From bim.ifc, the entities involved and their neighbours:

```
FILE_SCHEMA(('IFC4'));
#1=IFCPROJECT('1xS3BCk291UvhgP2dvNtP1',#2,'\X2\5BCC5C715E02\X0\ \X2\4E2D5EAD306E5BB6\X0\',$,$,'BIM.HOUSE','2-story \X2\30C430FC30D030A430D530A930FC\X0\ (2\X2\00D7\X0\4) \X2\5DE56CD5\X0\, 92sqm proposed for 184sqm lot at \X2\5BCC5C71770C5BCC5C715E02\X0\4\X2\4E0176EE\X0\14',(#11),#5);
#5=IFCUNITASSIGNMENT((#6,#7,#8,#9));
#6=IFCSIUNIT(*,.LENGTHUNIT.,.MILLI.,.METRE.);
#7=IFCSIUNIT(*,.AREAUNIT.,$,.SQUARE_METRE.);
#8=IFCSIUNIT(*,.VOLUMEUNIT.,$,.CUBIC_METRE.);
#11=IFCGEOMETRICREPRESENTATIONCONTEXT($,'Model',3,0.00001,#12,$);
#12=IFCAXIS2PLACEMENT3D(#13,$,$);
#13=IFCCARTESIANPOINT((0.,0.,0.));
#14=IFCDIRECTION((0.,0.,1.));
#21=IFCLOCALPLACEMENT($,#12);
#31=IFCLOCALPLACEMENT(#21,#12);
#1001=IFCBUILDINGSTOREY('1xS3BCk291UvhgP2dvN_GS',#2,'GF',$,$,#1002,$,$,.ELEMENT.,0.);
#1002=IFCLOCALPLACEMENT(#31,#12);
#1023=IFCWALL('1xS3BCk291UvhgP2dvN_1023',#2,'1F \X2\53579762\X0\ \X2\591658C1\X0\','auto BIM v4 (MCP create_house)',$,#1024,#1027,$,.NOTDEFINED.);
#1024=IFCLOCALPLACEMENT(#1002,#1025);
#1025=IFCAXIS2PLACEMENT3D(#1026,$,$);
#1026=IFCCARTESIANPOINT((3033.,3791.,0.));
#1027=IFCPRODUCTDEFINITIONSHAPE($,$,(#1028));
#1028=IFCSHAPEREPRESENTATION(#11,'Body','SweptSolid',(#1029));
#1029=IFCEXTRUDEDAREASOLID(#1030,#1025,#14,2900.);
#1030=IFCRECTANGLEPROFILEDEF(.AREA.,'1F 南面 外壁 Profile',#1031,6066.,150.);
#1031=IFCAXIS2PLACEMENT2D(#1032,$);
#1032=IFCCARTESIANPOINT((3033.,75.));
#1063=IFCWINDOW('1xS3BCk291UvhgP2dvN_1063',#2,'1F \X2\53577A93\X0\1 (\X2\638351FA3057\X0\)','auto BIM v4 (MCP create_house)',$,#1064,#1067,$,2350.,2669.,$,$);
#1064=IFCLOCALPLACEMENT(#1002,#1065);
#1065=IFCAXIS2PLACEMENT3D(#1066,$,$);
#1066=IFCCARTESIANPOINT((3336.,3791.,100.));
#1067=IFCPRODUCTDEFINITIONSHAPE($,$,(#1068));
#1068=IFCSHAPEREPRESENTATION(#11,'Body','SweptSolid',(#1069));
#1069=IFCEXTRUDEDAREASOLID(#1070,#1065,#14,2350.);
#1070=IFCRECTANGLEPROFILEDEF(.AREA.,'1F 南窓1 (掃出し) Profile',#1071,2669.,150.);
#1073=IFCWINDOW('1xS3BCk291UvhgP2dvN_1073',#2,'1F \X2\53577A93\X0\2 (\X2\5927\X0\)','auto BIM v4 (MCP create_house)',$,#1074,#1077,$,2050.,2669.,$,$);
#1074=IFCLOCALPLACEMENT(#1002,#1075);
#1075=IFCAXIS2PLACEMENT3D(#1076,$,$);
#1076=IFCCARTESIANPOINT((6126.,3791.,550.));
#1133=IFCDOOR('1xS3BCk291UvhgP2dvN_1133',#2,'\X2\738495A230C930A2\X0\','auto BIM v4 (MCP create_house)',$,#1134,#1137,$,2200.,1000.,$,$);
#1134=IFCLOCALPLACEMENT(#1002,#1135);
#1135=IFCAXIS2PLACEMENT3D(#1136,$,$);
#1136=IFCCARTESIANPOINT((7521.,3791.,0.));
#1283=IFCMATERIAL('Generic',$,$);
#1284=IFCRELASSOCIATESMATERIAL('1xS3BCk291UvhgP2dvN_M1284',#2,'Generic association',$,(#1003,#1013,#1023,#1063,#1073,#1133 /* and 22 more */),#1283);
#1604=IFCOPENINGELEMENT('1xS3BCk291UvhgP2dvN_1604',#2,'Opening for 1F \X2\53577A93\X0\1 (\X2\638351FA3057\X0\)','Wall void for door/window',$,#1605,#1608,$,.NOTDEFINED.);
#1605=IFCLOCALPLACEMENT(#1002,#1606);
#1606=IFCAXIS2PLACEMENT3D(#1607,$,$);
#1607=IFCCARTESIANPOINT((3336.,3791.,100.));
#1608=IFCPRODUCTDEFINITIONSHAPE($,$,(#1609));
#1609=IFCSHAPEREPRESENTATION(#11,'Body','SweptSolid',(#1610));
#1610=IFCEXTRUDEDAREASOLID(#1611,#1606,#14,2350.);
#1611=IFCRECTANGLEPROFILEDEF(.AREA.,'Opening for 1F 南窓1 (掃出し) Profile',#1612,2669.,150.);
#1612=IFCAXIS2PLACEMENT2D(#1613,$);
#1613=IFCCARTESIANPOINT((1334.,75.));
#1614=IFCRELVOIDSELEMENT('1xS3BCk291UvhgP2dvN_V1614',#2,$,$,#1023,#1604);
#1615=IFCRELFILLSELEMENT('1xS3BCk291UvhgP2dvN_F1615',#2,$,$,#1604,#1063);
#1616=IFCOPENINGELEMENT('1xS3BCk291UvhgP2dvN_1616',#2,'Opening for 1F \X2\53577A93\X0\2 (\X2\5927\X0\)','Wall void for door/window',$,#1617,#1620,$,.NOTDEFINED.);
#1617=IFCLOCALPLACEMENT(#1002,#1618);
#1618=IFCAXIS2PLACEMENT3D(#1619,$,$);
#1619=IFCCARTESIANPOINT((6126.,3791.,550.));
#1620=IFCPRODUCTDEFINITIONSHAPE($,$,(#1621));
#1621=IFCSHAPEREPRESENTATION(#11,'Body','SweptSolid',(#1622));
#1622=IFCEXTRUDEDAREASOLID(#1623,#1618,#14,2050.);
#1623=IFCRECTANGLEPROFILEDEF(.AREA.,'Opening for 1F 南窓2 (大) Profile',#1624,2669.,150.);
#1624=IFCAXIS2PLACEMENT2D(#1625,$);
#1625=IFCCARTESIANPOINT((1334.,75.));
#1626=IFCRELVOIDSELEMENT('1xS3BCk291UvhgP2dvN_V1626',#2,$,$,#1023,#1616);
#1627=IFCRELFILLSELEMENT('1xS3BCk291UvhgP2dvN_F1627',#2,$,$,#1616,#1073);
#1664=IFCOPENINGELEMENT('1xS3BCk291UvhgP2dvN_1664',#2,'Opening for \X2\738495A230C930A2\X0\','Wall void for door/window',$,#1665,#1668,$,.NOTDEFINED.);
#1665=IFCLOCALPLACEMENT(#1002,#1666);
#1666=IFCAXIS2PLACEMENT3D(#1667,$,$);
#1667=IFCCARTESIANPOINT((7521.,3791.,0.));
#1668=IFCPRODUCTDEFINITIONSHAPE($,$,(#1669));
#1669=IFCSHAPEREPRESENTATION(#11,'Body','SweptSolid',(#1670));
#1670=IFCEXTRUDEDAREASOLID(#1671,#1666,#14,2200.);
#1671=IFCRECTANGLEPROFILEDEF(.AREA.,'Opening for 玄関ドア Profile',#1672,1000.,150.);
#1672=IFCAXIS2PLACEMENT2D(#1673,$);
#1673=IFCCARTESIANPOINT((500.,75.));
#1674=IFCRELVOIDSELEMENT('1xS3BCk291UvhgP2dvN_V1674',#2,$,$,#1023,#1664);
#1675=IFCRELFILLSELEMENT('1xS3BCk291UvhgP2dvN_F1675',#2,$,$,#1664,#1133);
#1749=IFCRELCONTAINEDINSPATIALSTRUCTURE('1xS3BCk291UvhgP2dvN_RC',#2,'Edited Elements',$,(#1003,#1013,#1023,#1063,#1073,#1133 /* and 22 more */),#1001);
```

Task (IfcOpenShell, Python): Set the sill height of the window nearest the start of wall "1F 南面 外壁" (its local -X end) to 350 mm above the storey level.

```python
import numpy as np
import ifcopenshell
import ifcopenshell.api.geometry
import ifcopenshell.geom
import ifcopenshell.util.element
import ifcopenshell.util.placement
import ifcopenshell.util.shape
import ifcopenshell.util.unit

model = ifcopenshell.open("bim.ifc")
unit_scale = ifcopenshell.util.unit.calculate_unit_scale(model)

window = model.by_guid("1xS3BCk291UvhgP2dvN_1063")
opening = window.FillsVoids[0].RelatingOpeningElement
storey = ifcopenshell.util.element.get_container(window, ifc_class="IfcBuildingStorey")
level = ifcopenshell.util.placement.get_local_placement(storey.ObjectPlacement)[2, 3]

# The opening's origin need not be at the sill, so measure its lowest point.
shape = ifcopenshell.geom.create_shape(ifcopenshell.geom.settings(), opening)
bottom = ifcopenshell.util.shape.get_shape_bottom_elevation(shape, shape.geometry) / unit_scale
dz = level + 0.35 / unit_scale - bottom

shift = np.array([0.0, 0.0, dz])
# The window is not placed relative to its opening, so move both.
for product in (opening, window):
    matrix = ifcopenshell.util.placement.get_local_placement(product.ObjectPlacement)
    matrix[:3, 3] += shift
    ifcopenshell.api.geometry.edit_object_placement(model, product=product, matrix=matrix, is_si=False)

print(f"moved by {dz * unit_scale:+.3f} m")

model.write("bim_edited.ifc")
```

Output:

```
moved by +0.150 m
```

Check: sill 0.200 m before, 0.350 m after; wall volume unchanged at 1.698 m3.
